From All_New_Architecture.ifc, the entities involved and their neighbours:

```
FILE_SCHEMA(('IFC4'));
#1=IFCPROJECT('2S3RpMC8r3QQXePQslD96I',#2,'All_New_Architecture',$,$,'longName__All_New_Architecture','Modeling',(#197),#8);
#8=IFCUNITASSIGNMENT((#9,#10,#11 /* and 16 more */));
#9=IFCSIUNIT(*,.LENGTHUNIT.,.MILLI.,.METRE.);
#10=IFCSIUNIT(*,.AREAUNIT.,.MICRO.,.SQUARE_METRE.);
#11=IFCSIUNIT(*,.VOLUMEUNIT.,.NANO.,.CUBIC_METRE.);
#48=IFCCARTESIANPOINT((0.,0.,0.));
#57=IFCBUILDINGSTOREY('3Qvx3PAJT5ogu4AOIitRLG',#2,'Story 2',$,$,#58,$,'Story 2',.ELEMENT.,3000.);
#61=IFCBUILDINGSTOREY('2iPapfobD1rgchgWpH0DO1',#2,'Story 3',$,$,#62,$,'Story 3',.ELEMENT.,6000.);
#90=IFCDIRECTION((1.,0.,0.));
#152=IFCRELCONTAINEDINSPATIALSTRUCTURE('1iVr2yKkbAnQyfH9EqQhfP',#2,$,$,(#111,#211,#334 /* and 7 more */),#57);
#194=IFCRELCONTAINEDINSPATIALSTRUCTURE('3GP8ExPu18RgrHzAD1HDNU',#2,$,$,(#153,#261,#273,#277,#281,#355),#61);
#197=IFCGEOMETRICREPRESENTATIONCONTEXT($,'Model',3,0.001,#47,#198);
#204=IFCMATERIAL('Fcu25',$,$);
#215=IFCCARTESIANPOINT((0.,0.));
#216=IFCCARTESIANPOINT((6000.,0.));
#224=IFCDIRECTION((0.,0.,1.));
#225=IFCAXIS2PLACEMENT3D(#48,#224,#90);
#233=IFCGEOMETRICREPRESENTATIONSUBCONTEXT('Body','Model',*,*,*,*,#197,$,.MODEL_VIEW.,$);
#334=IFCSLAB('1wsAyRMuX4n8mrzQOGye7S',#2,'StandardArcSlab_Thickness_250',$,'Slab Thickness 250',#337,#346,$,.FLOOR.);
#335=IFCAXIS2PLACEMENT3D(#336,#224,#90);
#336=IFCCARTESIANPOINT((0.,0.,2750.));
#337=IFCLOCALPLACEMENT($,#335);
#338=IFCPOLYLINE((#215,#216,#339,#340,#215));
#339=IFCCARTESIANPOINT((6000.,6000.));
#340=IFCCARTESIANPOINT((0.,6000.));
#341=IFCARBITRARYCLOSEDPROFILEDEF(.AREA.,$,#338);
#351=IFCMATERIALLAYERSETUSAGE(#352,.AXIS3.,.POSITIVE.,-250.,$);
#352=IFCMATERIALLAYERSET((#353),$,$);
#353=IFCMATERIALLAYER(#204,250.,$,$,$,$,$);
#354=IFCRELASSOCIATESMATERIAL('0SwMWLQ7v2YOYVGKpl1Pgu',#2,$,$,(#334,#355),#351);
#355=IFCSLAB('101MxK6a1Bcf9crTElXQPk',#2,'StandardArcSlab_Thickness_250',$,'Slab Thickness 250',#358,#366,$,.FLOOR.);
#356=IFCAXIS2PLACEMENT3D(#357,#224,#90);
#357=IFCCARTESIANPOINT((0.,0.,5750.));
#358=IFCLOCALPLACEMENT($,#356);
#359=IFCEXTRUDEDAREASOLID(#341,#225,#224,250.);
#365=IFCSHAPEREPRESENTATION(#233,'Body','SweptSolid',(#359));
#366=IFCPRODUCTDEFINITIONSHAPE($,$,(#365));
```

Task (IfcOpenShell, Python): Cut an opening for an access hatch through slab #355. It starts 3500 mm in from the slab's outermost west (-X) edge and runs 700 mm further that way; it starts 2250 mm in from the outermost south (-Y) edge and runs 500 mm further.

```python
import numpy as np
import ifcopenshell
import ifcopenshell.api.feature
import ifcopenshell.api.geometry
import ifcopenshell.api.root
import ifcopenshell.geom
import ifcopenshell.util.placement
import ifcopenshell.util.representation
import ifcopenshell.util.shape
import ifcopenshell.util.unit

model = ifcopenshell.open("All_New_Architecture.ifc")
unit_scale = ifcopenshell.util.unit.calculate_unit_scale(model)
settings = ifcopenshell.geom.settings()


def volume(element):
    """Net volume in cubic metres, openings subtracted."""
    shape = ifcopenshell.geom.create_shape(settings, element)
    return ifcopenshell.util.shape.get_volume(shape.geometry)


slab = model.by_id(355)
before = volume(slab)

# Extent in the slab's own axes, in metres. The edges named are its -X and -Y sides.
slab_shape = ifcopenshell.geom.create_shape(settings, slab)
vertices = ifcopenshell.util.shape.get_vertices(slab_shape.geometry)
x_min, y_min, bottom = vertices.min(axis=0)
top = vertices[:, 2].max()

opening = ifcopenshell.api.root.create_entity(model, ifc_class="IfcOpeningElement", name="Access hatch opening", predefined_type="OPENING")
context = ifcopenshell.util.representation.get_context(model, "Model", "Body", "MODEL_VIEW")
width, depth = 0.7, 0.5
outline = [(0.0, 0.0), (width, 0.0), (width, depth), (0.0, depth), (0.0, 0.0)]
# Overshoot both faces by 50 mm so the cut is clean.
shape = ifcopenshell.api.geometry.add_slab_representation(
    model, context=context, depth=top - bottom + 0.1, polyline=outline
)
ifcopenshell.api.geometry.assign_representation(model, product=opening, representation=shape)

matrix = ifcopenshell.util.placement.get_local_placement(slab.ObjectPlacement)
matrix[:, 3] = matrix @ np.append(np.array([x_min + 3.5, y_min + 2.25, bottom - 0.05]) / unit_scale, 1.0)
ifcopenshell.api.geometry.edit_object_placement(model, product=opening, matrix=matrix, is_si=False)
ifcopenshell.api.feature.add_feature(model, feature=opening, element=slab)

after = volume(slab)

print(f"slab volume {before:.3f} -> {after:.3f} m3")

model.write("All_New_Architecture_rev.ifc")
```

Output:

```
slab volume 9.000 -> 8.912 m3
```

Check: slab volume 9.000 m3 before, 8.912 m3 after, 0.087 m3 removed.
